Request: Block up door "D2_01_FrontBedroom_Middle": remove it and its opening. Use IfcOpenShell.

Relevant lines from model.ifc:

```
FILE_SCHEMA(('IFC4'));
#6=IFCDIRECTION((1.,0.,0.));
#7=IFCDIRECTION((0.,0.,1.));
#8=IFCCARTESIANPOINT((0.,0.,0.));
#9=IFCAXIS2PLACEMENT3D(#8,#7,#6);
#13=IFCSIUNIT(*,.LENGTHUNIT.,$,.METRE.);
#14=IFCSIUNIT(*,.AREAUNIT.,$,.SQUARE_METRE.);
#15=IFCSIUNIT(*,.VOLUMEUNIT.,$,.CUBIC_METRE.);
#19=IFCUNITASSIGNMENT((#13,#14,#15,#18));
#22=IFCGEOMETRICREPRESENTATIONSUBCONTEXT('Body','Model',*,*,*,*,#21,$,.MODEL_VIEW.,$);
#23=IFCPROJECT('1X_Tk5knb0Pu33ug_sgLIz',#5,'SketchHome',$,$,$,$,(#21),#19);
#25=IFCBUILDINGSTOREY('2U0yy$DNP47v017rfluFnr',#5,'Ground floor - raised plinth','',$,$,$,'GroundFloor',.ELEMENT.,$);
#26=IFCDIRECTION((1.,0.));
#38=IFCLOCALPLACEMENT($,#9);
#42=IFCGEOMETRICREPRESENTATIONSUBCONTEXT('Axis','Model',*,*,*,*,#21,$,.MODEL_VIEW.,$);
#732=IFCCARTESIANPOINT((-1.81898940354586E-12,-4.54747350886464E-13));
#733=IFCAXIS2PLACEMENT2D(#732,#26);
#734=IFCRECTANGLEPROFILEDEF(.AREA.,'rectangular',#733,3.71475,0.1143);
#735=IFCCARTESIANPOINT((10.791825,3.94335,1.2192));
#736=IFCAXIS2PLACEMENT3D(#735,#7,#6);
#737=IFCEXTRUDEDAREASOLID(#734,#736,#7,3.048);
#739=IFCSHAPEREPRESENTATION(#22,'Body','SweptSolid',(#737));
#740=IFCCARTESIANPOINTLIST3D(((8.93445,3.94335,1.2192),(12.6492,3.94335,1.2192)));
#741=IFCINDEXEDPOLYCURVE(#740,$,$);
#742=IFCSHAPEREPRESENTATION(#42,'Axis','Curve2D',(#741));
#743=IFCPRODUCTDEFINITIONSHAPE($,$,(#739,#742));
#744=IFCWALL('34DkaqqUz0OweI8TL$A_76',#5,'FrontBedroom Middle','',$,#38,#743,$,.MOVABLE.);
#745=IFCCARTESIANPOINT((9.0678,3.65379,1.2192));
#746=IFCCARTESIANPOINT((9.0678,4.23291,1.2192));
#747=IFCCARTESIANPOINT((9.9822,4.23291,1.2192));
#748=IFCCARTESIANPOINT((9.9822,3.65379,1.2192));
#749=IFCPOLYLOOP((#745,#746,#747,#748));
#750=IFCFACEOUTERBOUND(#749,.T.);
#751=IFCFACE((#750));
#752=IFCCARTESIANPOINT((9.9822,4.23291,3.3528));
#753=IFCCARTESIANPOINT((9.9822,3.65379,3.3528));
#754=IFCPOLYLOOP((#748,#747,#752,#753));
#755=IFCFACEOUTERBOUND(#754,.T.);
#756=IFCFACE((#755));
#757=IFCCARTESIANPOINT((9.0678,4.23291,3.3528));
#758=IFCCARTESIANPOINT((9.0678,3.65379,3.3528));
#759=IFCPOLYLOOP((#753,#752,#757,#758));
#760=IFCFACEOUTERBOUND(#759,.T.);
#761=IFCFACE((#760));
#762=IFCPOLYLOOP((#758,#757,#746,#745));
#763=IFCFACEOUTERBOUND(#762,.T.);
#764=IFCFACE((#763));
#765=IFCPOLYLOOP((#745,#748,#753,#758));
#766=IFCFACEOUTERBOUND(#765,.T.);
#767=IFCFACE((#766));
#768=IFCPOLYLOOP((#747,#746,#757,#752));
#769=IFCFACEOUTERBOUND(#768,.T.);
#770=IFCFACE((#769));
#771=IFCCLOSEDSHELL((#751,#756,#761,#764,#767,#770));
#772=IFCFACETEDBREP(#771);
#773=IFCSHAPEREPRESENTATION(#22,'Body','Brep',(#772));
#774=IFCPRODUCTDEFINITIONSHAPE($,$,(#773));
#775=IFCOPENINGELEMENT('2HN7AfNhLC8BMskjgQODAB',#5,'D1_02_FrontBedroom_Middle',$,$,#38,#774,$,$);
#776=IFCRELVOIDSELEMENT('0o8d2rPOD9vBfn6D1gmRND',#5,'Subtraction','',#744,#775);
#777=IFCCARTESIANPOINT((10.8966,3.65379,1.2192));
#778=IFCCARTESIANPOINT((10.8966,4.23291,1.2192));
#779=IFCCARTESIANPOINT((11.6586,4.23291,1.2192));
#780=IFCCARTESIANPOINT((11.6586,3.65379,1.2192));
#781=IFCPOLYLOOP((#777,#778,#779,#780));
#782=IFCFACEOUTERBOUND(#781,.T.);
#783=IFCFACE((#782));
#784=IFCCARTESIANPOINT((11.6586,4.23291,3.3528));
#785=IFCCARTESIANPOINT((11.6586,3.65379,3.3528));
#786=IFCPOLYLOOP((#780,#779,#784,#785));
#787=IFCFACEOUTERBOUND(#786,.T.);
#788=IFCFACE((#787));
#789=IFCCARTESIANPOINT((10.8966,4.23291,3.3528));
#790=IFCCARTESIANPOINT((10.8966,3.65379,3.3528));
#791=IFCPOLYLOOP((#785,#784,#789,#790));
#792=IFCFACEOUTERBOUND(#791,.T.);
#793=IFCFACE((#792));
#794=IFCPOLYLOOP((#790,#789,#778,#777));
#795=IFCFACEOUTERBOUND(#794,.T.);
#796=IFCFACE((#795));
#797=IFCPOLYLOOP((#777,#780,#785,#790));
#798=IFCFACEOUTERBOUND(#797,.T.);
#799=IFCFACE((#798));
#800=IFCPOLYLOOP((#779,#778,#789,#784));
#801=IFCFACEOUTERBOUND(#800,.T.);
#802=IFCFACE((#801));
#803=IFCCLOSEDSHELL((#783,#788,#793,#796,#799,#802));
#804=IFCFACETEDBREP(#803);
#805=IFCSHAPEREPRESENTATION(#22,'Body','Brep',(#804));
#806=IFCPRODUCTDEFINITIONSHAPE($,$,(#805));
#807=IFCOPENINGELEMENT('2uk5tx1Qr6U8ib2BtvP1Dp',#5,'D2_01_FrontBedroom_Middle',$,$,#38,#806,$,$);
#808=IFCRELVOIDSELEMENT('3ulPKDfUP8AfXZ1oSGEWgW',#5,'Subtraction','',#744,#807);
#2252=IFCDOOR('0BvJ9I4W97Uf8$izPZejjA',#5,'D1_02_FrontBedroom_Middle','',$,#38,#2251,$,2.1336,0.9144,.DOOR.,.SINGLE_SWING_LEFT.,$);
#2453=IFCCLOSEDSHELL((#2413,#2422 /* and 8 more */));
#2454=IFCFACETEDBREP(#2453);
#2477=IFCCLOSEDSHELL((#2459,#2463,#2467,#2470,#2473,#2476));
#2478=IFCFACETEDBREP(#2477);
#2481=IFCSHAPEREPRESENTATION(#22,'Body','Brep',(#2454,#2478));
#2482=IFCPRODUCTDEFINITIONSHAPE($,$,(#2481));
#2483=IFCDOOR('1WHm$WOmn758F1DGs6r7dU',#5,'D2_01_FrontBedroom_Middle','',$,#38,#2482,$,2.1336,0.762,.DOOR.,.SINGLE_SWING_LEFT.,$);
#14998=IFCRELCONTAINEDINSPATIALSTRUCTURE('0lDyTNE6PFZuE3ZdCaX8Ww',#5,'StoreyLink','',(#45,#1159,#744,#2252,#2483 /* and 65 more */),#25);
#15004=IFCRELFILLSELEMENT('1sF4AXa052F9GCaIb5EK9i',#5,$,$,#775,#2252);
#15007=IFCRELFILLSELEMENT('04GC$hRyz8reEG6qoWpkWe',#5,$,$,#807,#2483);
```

```python
import ifcopenshell
import ifcopenshell.api.feature
import ifcopenshell.api.root
import ifcopenshell.geom
import ifcopenshell.util.shape

model = ifcopenshell.open("model.ifc")
settings = ifcopenshell.geom.settings()


def volume(element):
    """Net volume in cubic metres, openings subtracted."""
    shape = ifcopenshell.geom.create_shape(settings, element)
    return ifcopenshell.util.shape.get_volume(shape.geometry)


door = model.by_id(2483)
opening = door.FillsVoids[0].RelatingOpeningElement
wall = opening.VoidsElements[0].RelatingBuildingElement
before = volume(wall)

ifcopenshell.api.root.remove_product(model, product=door)
ifcopenshell.api.feature.remove_feature(model, feature=opening)

after = volume(wall)

print(f"wall volume {before:.3f} -> {after:.3f} m3")

model.write("model_edited.ifc")
```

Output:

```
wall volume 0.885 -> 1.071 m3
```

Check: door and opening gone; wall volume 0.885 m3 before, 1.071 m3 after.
